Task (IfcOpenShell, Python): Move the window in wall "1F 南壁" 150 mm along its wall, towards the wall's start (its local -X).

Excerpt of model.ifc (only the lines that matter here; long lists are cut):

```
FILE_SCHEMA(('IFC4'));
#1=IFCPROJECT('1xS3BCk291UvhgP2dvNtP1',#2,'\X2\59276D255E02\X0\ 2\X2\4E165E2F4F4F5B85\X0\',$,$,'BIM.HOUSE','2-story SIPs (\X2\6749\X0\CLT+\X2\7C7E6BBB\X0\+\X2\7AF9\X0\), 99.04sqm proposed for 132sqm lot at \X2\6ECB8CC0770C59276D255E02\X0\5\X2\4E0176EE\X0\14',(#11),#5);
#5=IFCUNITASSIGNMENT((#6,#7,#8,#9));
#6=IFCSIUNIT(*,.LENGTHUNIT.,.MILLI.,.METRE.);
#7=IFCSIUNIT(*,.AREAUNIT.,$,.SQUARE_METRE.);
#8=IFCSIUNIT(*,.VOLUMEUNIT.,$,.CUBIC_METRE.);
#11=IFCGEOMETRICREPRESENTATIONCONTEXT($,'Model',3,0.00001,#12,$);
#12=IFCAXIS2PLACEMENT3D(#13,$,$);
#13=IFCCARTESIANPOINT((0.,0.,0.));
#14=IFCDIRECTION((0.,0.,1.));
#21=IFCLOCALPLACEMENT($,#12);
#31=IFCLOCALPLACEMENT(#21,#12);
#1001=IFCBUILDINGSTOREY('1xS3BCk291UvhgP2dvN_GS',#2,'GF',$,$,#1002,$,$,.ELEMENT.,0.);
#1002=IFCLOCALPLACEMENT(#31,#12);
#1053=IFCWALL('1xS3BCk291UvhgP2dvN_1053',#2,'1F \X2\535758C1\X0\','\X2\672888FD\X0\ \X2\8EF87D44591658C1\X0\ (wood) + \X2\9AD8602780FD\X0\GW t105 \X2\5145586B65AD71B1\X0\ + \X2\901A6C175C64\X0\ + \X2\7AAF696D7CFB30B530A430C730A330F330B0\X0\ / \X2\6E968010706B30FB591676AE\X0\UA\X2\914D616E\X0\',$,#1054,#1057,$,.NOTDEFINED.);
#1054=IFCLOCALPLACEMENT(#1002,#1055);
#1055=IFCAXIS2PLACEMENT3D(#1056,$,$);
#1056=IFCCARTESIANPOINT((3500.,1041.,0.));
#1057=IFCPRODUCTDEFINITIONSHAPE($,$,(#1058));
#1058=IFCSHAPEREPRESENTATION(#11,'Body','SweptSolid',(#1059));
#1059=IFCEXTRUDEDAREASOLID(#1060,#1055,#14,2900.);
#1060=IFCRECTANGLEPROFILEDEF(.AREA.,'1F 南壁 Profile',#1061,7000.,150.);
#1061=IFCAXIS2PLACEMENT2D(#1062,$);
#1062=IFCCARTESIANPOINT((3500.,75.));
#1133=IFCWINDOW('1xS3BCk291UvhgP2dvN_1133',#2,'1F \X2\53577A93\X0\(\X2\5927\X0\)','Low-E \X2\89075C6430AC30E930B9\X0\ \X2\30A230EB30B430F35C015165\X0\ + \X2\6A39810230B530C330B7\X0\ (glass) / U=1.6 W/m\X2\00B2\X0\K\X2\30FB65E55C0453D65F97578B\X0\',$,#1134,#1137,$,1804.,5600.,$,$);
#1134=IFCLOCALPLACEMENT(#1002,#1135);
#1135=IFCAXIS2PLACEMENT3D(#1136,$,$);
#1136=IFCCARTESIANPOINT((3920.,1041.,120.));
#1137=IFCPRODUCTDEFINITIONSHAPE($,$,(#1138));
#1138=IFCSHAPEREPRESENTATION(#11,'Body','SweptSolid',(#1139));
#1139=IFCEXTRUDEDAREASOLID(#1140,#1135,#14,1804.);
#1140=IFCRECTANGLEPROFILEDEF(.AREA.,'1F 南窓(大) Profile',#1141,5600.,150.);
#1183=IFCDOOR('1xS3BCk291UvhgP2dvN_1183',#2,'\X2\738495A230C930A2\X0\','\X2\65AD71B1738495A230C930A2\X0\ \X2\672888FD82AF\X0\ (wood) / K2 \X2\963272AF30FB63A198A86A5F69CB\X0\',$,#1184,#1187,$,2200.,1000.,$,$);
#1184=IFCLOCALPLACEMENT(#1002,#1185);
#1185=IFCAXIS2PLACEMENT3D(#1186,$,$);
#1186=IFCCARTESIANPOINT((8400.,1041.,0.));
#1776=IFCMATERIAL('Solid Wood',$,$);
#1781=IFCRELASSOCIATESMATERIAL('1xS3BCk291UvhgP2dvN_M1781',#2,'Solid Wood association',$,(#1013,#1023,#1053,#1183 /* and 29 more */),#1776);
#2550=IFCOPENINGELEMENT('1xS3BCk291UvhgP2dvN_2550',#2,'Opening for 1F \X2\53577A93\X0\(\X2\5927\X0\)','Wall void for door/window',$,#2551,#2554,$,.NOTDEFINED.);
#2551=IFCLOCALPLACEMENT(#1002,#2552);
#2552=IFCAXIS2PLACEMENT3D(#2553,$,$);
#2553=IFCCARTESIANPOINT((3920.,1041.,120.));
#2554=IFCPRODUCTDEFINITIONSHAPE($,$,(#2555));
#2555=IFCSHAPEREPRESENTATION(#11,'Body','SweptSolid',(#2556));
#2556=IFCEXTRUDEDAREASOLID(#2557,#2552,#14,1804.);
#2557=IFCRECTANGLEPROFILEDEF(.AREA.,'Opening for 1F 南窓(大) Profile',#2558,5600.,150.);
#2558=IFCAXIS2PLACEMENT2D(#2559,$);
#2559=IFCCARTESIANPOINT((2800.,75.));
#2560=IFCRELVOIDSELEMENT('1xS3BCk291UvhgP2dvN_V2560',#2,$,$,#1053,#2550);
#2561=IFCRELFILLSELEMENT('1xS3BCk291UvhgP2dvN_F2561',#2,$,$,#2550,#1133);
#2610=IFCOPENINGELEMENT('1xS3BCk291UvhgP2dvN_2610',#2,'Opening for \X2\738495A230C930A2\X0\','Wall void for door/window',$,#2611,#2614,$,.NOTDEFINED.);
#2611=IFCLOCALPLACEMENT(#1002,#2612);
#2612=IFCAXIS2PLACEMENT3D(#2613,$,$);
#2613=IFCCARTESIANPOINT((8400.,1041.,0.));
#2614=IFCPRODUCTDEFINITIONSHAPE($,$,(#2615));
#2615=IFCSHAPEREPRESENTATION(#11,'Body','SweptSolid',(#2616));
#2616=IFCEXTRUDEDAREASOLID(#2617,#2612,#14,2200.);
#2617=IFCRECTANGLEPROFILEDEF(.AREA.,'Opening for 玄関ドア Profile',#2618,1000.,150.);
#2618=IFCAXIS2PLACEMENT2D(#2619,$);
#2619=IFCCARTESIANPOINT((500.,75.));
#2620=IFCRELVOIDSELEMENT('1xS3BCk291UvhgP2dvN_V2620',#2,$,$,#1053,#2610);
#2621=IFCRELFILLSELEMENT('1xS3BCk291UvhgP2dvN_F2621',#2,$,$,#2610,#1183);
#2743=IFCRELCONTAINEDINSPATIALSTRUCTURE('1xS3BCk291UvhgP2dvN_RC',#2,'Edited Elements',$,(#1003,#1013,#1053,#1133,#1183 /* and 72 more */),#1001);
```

```python
import ifcopenshell
import ifcopenshell.api.geometry
import ifcopenshell.util.placement

model = ifcopenshell.open("model.ifc")

window = model.by_id(1133)
opening = window.FillsVoids[0].RelatingOpeningElement
wall = opening.VoidsElements[0].RelatingBuildingElement

wall_matrix = ifcopenshell.util.placement.get_local_placement(wall.ObjectPlacement)
shift = wall_matrix[:3, 0] * -150.0
before = ifcopenshell.util.placement.get_local_placement(window.ObjectPlacement)[:3, 3].copy()

# The window is not placed relative to its opening, so move both.
for product in (opening, window):
    matrix = ifcopenshell.util.placement.get_local_placement(product.ObjectPlacement)
    matrix[:3, 3] += shift
    ifcopenshell.api.geometry.edit_object_placement(model, product=product, matrix=matrix, is_si=False)

after = ifcopenshell.util.placement.get_local_placement(window.ObjectPlacement)[:3, 3]
print("window moved by", (after - before).round(3) + 0.0)

model.write("model-out.ifc")
```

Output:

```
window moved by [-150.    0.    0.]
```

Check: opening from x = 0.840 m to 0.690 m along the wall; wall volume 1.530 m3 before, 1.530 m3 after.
